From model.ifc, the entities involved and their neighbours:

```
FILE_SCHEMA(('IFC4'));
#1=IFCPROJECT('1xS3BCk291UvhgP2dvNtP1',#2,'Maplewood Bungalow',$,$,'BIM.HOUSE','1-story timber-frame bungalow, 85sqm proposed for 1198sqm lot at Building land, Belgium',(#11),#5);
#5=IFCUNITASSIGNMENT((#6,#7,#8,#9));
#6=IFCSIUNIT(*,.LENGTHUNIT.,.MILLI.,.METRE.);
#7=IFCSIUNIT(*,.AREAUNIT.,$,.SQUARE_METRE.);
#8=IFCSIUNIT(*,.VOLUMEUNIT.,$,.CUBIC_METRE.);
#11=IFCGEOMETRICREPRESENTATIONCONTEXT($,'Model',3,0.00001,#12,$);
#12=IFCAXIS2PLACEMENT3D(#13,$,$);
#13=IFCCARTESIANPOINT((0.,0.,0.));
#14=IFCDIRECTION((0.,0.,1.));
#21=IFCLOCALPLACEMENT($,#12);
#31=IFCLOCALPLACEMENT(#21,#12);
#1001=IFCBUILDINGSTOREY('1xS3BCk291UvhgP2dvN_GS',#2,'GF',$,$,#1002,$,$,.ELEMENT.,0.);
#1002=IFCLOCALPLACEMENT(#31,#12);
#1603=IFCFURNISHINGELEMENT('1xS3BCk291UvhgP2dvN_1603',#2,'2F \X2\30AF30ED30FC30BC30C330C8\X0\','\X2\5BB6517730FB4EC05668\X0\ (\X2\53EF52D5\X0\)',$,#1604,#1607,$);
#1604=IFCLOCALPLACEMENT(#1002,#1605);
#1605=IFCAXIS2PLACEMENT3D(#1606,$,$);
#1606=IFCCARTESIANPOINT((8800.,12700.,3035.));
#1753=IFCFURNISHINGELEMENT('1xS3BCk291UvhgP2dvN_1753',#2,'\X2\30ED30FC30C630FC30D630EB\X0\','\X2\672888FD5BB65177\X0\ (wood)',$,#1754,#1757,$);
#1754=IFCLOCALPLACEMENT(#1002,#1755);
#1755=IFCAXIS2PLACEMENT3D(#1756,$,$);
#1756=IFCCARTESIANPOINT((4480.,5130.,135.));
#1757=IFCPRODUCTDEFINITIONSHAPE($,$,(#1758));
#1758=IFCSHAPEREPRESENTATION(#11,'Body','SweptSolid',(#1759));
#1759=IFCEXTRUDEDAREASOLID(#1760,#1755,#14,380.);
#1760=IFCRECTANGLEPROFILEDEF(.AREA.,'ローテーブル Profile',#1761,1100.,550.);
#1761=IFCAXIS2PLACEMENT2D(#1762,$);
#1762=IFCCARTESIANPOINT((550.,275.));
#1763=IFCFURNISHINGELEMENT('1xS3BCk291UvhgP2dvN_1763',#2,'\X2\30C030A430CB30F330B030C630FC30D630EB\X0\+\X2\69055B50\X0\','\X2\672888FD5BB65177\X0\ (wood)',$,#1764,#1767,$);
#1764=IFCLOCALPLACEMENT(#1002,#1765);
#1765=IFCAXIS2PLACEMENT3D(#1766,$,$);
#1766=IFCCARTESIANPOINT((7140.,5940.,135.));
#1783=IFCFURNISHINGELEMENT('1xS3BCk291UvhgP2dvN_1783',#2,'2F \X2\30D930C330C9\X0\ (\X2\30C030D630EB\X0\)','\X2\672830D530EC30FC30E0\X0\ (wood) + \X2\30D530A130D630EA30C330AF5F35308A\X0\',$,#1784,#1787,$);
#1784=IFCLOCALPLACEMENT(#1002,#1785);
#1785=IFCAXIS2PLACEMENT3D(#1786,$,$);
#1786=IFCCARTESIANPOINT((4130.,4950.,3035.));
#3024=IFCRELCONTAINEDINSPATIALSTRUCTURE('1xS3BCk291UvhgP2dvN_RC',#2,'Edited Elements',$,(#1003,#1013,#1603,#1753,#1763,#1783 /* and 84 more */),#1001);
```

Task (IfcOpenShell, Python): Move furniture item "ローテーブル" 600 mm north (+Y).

```python
import ifcopenshell
import ifcopenshell.api.geometry
import ifcopenshell.util.placement

model = ifcopenshell.open("model.ifc")

item = model.by_id(1753)
matrix = ifcopenshell.util.placement.get_local_placement(item.ObjectPlacement)
matrix[1, 3] += 600.0
ifcopenshell.api.geometry.edit_object_placement(model, product=item, matrix=matrix, is_si=False)

print(ifcopenshell.util.placement.get_local_placement(item.ObjectPlacement).round(3) + 0.0)

model.write("model_updated.ifc")
```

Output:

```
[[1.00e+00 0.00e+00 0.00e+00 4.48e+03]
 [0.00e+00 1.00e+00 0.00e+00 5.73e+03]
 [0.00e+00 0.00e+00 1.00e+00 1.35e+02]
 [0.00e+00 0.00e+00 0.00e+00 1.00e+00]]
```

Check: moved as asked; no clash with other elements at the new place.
